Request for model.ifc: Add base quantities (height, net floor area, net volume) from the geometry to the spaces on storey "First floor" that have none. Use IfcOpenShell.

First a look at what the model holds.

```python
import ifcopenshell
import ifcopenshell.util.element
import ifcopenshell.util.unit

model = ifcopenshell.open("model.ifc")
print(model.schema)
for unit_type in ("LENGTHUNIT", "AREAUNIT", "VOLUMEUNIT"):
    print(unit_type, ifcopenshell.util.unit.calculate_unit_scale(model, unit_type))
storey = next(s for s in model.by_type("IfcBuildingStorey") if s.Name == "First floor")
spaces = [e for e in ifcopenshell.util.element.get_decomposition(storey) if e.is_a("IfcSpace")]
for e in sorted(spaces, key=lambda e: e.id()):
    print(e.id(), e.is_a(), e.Name, list(ifcopenshell.util.element.get_psets(e, qtos_only=True)), sep=" | ")
```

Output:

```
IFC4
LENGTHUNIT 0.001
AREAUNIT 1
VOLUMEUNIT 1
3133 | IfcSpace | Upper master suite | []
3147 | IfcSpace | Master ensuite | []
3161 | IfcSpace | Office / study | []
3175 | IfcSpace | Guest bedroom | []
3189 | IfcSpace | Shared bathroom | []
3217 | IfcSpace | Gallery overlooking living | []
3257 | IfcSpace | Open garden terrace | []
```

```python
import ifcopenshell
import ifcopenshell.api.pset
import ifcopenshell.geom
import ifcopenshell.util.element
import ifcopenshell.util.shape
import ifcopenshell.util.unit

model = ifcopenshell.open("model.ifc")
unit_scale = ifcopenshell.util.unit.calculate_unit_scale(model)
area_scale = ifcopenshell.util.unit.calculate_unit_scale(model, "AREAUNIT")
volume_scale = ifcopenshell.util.unit.calculate_unit_scale(model, "VOLUMEUNIT")
settings = ifcopenshell.geom.settings()

storey = next(s for s in model.by_type("IfcBuildingStorey") if s.Name == "First floor")
spaces = [e for e in ifcopenshell.util.element.get_decomposition(storey) if e.is_a("IfcSpace")]

for e in sorted(spaces, key=lambda e: e.id()):
    if ifcopenshell.util.element.get_psets(e, qtos_only=True, should_inherit=False):
        continue
    # Geometry comes back in metres, in the element's own axes.
    shape = ifcopenshell.geom.create_shape(settings, e)
    values = {
        "Height": ifcopenshell.util.shape.get_z(shape.geometry) / unit_scale,
        "NetFloorArea": ifcopenshell.util.shape.get_footprint_area(shape.geometry) / area_scale,
        "NetVolume": ifcopenshell.util.shape.get_volume(shape.geometry) / volume_scale,
    }
    qto = ifcopenshell.api.pset.add_qto(model, product=e, name="Qto_SpaceBaseQuantities")
    ifcopenshell.api.pset.edit_qto(model, qto=qto, properties=values)
    print(e.id(), {k: round(v, 3) for k, v in values.items()})

model.write("model-out.ifc")
```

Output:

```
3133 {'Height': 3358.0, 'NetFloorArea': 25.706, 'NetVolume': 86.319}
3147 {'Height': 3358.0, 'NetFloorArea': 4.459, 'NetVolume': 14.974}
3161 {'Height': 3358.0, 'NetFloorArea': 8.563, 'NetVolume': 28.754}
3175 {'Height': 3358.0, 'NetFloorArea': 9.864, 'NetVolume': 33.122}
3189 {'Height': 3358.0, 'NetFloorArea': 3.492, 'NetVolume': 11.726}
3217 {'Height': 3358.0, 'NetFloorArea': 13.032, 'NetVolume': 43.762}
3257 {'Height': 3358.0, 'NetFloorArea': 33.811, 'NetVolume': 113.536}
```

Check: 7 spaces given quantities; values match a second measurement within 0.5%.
